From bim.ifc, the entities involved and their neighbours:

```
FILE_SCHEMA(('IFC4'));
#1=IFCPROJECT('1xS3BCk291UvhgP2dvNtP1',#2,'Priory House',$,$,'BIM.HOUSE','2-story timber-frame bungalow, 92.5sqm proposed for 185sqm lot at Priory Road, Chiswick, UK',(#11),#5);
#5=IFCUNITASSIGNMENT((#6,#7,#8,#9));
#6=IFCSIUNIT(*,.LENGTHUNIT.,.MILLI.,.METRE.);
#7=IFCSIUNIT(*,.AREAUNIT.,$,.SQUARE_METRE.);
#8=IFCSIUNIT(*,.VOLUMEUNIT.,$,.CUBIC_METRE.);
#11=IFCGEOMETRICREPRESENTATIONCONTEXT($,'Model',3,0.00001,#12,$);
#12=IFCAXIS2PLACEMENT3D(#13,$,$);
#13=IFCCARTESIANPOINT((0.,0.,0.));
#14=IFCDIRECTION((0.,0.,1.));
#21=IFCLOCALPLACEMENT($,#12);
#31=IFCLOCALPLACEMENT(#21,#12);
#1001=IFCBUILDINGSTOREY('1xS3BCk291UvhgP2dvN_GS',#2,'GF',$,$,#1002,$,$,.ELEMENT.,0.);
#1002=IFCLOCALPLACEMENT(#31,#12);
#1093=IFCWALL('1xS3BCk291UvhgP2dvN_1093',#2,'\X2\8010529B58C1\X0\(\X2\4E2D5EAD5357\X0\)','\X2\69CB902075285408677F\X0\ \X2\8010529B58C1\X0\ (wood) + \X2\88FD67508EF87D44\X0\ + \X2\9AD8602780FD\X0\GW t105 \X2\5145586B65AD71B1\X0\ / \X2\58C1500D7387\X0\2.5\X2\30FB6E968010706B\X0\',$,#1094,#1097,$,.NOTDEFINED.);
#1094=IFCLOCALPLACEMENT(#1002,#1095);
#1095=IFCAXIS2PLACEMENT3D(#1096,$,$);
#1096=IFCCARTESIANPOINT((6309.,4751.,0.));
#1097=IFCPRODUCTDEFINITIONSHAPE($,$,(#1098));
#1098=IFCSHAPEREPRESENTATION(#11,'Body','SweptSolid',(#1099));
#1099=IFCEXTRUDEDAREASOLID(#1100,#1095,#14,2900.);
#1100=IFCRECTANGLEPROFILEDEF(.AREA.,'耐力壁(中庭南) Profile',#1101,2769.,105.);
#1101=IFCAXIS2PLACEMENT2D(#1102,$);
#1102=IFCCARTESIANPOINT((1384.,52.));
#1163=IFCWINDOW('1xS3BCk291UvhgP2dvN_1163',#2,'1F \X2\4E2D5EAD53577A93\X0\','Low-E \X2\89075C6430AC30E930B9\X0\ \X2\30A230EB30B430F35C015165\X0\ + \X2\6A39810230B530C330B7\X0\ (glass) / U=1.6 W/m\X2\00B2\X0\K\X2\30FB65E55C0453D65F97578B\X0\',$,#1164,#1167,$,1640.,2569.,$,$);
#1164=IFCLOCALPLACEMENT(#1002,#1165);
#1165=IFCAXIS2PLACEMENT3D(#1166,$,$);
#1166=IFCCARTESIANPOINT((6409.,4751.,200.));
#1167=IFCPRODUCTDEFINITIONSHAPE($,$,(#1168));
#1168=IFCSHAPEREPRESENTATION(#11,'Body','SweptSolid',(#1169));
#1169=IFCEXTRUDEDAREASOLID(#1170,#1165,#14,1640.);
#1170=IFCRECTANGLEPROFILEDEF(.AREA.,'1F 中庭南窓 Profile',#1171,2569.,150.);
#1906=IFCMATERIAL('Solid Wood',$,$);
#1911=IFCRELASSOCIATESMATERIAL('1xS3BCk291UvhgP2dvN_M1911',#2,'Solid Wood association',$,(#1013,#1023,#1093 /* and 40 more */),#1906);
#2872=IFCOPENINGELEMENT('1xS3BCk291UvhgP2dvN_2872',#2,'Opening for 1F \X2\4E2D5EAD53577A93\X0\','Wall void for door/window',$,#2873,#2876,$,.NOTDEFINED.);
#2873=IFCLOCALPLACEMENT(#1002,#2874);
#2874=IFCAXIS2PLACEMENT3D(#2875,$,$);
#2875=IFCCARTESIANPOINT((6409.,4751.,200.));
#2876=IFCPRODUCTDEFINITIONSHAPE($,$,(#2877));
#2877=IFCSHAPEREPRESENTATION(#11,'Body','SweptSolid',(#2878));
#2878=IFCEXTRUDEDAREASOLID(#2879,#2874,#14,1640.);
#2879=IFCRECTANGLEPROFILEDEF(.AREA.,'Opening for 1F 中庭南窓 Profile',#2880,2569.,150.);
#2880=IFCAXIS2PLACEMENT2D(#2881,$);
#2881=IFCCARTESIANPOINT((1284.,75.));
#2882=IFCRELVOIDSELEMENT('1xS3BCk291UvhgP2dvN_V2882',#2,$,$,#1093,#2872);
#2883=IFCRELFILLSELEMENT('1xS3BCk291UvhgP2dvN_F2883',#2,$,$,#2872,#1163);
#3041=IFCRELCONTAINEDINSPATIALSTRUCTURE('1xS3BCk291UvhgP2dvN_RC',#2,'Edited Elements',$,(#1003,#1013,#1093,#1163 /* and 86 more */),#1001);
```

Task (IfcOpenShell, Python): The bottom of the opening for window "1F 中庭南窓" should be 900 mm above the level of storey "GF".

```python
import numpy as np
import ifcopenshell
import ifcopenshell.api.geometry
import ifcopenshell.geom
import ifcopenshell.util.element
import ifcopenshell.util.placement
import ifcopenshell.util.shape
import ifcopenshell.util.unit

model = ifcopenshell.open("bim.ifc")
unit_scale = ifcopenshell.util.unit.calculate_unit_scale(model)

window = model.by_guid("1xS3BCk291UvhgP2dvN_1163")
opening = window.FillsVoids[0].RelatingOpeningElement
storey = ifcopenshell.util.element.get_container(window, ifc_class="IfcBuildingStorey")
level = ifcopenshell.util.placement.get_local_placement(storey.ObjectPlacement)[2, 3]

# The opening's origin need not be at the sill, so measure its lowest point.
shape = ifcopenshell.geom.create_shape(ifcopenshell.geom.settings(), opening)
bottom = ifcopenshell.util.shape.get_shape_bottom_elevation(shape, shape.geometry) / unit_scale
dz = level + 900.0 - bottom

shift = np.array([0.0, 0.0, dz])
# The window is not placed relative to its opening, so move both.
for product in (opening, window):
    matrix = ifcopenshell.util.placement.get_local_placement(product.ObjectPlacement)
    matrix[:3, 3] += shift
    ifcopenshell.api.geometry.edit_object_placement(model, product=product, matrix=matrix, is_si=False)

print(f"moved by {dz * unit_scale:+.3f} m")

model.write("bim_edited.ifc")
```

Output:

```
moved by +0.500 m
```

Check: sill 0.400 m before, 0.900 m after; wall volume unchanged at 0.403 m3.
